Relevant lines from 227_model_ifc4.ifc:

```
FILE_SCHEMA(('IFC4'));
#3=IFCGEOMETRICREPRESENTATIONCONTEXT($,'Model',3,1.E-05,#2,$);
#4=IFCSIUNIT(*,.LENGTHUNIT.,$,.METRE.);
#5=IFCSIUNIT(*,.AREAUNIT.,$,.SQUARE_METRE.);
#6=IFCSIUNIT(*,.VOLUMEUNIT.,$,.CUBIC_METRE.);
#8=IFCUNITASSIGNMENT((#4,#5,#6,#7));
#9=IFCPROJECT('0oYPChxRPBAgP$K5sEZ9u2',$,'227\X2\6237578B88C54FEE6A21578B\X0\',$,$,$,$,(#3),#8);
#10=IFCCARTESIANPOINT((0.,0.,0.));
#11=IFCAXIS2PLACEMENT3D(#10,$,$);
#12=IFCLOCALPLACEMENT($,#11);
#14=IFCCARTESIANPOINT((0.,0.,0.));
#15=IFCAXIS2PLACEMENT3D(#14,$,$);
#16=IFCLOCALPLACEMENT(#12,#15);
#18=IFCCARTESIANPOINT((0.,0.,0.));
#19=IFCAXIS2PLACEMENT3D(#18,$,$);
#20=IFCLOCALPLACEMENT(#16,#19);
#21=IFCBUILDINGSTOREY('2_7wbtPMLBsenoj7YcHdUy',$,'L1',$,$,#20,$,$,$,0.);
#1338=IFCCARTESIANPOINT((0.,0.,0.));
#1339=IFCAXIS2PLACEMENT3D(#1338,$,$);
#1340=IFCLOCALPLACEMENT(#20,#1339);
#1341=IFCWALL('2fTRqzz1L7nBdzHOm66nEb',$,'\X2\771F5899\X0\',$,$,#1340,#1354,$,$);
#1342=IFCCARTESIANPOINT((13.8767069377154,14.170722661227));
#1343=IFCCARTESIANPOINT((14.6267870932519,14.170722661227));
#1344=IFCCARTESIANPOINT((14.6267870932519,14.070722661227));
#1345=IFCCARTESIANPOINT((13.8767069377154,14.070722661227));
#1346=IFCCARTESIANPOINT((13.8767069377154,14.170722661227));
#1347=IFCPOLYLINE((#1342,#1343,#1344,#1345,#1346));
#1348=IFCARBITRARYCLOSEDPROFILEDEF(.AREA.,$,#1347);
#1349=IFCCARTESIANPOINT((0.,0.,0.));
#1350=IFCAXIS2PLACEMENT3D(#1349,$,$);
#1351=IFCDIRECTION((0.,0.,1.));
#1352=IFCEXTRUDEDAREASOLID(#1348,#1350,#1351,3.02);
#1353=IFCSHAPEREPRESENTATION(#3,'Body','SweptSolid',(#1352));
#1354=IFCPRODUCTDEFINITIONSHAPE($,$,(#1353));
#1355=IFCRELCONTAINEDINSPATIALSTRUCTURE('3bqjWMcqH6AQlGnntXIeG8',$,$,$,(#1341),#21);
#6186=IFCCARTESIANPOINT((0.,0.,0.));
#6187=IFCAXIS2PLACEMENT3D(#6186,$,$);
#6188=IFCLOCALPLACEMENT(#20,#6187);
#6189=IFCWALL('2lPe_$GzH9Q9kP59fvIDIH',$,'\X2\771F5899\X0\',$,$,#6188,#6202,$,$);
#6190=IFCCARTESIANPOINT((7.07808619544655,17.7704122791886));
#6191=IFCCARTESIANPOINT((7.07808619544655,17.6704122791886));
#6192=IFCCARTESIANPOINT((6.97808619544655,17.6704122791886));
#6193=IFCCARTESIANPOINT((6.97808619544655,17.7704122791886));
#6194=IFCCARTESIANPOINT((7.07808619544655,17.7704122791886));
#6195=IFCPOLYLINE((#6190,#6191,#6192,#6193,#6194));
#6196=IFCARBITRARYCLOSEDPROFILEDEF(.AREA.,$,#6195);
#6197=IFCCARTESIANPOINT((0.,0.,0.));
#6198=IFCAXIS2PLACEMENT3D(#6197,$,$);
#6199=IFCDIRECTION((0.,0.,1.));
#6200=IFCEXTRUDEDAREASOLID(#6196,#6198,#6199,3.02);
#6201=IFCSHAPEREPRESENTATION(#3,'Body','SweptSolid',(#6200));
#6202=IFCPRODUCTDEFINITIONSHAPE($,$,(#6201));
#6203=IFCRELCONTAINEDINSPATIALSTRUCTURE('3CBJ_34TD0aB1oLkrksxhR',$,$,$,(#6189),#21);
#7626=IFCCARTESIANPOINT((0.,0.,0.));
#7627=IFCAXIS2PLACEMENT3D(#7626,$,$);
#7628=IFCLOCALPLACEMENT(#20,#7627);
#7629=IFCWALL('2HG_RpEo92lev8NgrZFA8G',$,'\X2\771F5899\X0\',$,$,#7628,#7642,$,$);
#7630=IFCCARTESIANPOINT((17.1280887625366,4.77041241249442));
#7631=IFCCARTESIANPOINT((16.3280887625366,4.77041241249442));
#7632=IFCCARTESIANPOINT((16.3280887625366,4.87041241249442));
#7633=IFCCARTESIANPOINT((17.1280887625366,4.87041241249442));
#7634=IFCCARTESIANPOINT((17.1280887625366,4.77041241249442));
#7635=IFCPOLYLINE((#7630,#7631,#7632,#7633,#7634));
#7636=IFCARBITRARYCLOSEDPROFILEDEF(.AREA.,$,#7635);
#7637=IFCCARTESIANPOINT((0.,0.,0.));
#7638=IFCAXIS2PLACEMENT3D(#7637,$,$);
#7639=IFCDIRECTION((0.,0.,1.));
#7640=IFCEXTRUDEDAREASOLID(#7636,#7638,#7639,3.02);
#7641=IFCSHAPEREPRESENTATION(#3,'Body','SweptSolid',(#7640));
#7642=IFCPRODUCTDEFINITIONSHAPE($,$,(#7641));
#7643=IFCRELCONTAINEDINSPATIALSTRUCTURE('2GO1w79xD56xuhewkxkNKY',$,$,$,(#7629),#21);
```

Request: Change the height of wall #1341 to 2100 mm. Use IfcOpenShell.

```python
import ifcopenshell
import ifcopenshell.geom
import ifcopenshell.util.shape
import ifcopenshell.util.unit

model = ifcopenshell.open("227_model_ifc4.ifc")
unit_scale = ifcopenshell.util.unit.calculate_unit_scale(model)
settings = ifcopenshell.geom.settings()


def volume(element):
    """Net volume in cubic metres, openings subtracted."""
    shape = ifcopenshell.geom.create_shape(settings, element)
    return ifcopenshell.util.shape.get_volume(shape.geometry)


wall = model.by_id(1341)
before = volume(wall)

body = next(r for r in wall.Representation.Representations if r.RepresentationIdentifier == "Body")
solid = body.Items[0]
old_height = solid.Depth
solid.Depth = 2.1 / unit_scale
after = volume(wall)

print(f"height {old_height:g} -> {solid.Depth:g}, volume {before:.3f} -> {after:.3f} m3")

model.write("227_model_ifc4_updated.ifc")
```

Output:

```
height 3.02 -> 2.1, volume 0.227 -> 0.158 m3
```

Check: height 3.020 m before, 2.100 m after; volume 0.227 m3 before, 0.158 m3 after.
